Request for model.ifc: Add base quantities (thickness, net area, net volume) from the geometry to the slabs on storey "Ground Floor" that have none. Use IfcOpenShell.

First a look at what the model holds.

```python
import ifcopenshell
import ifcopenshell.util.element
import ifcopenshell.util.unit

model = ifcopenshell.open("model.ifc")
print(model.schema)
for unit_type in ("LENGTHUNIT", "AREAUNIT", "VOLUMEUNIT"):
    print(unit_type, ifcopenshell.util.unit.calculate_unit_scale(model, unit_type))
storey = next(s for s in model.by_type("IfcBuildingStorey") if s.Name == "Ground Floor")
slabs = [e for e in ifcopenshell.util.element.get_decomposition(storey) if e.is_a("IfcSlab")]
for e in sorted(slabs, key=lambda e: e.id()):
    print(e.id(), e.is_a(), e.Name, list(ifcopenshell.util.element.get_psets(e, qtos_only=True)), sep=" | ")
```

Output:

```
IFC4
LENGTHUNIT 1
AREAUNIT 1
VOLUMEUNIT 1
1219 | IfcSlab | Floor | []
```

```python
import ifcopenshell
import ifcopenshell.api.pset
import ifcopenshell.geom
import ifcopenshell.util.element
import ifcopenshell.util.shape
import ifcopenshell.util.unit

model = ifcopenshell.open("model.ifc")
unit_scale = ifcopenshell.util.unit.calculate_unit_scale(model)
area_scale = ifcopenshell.util.unit.calculate_unit_scale(model, "AREAUNIT")
volume_scale = ifcopenshell.util.unit.calculate_unit_scale(model, "VOLUMEUNIT")
settings = ifcopenshell.geom.settings()

storey = next(s for s in model.by_type("IfcBuildingStorey") if s.Name == "Ground Floor")
slabs = [e for e in ifcopenshell.util.element.get_decomposition(storey) if e.is_a("IfcSlab")]

for e in sorted(slabs, key=lambda e: e.id()):
    if ifcopenshell.util.element.get_psets(e, qtos_only=True, should_inherit=False):
        continue
    # Geometry comes back in metres, in the element's own axes.
    shape = ifcopenshell.geom.create_shape(settings, e)
    values = {
        "Width": ifcopenshell.util.shape.get_z(shape.geometry) / unit_scale,
        "NetArea": ifcopenshell.util.shape.get_footprint_area(shape.geometry) / area_scale,
        "NetVolume": ifcopenshell.util.shape.get_volume(shape.geometry) / volume_scale,
    }
    qto = ifcopenshell.api.pset.add_qto(model, product=e, name="Qto_SlabBaseQuantities")
    ifcopenshell.api.pset.edit_qto(model, qto=qto, properties=values)
    print(e.id(), {k: round(v, 3) for k, v in values.items()})

model.write("model_rev.ifc")
```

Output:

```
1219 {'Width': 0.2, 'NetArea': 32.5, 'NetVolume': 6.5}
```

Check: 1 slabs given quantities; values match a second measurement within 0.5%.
